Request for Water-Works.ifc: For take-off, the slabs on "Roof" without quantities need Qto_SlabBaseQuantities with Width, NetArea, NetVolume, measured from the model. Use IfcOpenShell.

First a look at what the model holds.

```python
import ifcopenshell
import ifcopenshell.util.element
import ifcopenshell.util.unit

model = ifcopenshell.open("Water-Works.ifc")
print(model.schema)
for unit_type in ("LENGTHUNIT", "AREAUNIT", "VOLUMEUNIT"):
    print(unit_type, ifcopenshell.util.unit.calculate_unit_scale(model, unit_type))
storey = next(s for s in model.by_type("IfcBuildingStorey") if s.Name == "Roof")
slabs = [e for e in ifcopenshell.util.element.get_decomposition(storey) if e.is_a("IfcSlab")]
for e in sorted(slabs, key=lambda e: e.id()):
    print(e.id(), e.is_a(), e.Name, list(ifcopenshell.util.element.get_psets(e, qtos_only=True)), sep=" | ")
```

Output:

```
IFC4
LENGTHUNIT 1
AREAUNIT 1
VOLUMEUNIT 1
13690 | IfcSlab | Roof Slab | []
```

```python
import ifcopenshell
import ifcopenshell.api.pset
import ifcopenshell.geom
import ifcopenshell.util.element
import ifcopenshell.util.shape
import ifcopenshell.util.unit

model = ifcopenshell.open("Water-Works.ifc")
unit_scale = ifcopenshell.util.unit.calculate_unit_scale(model)
area_scale = ifcopenshell.util.unit.calculate_unit_scale(model, "AREAUNIT")
volume_scale = ifcopenshell.util.unit.calculate_unit_scale(model, "VOLUMEUNIT")
settings = ifcopenshell.geom.settings()

storey = next(s for s in model.by_type("IfcBuildingStorey") if s.Name == "Roof")
slabs = [e for e in ifcopenshell.util.element.get_decomposition(storey) if e.is_a("IfcSlab")]

for e in sorted(slabs, key=lambda e: e.id()):
    if ifcopenshell.util.element.get_psets(e, qtos_only=True, should_inherit=False):
        continue
    # Geometry comes back in metres, in the element's own axes.
    shape = ifcopenshell.geom.create_shape(settings, e)
    values = {
        "Width": ifcopenshell.util.shape.get_z(shape.geometry) / unit_scale,
        "NetArea": ifcopenshell.util.shape.get_footprint_area(shape.geometry) / area_scale,
        "NetVolume": ifcopenshell.util.shape.get_volume(shape.geometry) / volume_scale,
    }
    qto = ifcopenshell.api.pset.add_qto(model, product=e, name="Qto_SlabBaseQuantities")
    ifcopenshell.api.pset.edit_qto(model, qto=qto, properties=values)
    print(e.id(), {k: round(v, 3) for k, v in values.items()})

model.write("Water-Works_edited.ifc")
```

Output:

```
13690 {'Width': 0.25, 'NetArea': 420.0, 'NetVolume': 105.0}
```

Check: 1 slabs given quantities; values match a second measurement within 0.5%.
